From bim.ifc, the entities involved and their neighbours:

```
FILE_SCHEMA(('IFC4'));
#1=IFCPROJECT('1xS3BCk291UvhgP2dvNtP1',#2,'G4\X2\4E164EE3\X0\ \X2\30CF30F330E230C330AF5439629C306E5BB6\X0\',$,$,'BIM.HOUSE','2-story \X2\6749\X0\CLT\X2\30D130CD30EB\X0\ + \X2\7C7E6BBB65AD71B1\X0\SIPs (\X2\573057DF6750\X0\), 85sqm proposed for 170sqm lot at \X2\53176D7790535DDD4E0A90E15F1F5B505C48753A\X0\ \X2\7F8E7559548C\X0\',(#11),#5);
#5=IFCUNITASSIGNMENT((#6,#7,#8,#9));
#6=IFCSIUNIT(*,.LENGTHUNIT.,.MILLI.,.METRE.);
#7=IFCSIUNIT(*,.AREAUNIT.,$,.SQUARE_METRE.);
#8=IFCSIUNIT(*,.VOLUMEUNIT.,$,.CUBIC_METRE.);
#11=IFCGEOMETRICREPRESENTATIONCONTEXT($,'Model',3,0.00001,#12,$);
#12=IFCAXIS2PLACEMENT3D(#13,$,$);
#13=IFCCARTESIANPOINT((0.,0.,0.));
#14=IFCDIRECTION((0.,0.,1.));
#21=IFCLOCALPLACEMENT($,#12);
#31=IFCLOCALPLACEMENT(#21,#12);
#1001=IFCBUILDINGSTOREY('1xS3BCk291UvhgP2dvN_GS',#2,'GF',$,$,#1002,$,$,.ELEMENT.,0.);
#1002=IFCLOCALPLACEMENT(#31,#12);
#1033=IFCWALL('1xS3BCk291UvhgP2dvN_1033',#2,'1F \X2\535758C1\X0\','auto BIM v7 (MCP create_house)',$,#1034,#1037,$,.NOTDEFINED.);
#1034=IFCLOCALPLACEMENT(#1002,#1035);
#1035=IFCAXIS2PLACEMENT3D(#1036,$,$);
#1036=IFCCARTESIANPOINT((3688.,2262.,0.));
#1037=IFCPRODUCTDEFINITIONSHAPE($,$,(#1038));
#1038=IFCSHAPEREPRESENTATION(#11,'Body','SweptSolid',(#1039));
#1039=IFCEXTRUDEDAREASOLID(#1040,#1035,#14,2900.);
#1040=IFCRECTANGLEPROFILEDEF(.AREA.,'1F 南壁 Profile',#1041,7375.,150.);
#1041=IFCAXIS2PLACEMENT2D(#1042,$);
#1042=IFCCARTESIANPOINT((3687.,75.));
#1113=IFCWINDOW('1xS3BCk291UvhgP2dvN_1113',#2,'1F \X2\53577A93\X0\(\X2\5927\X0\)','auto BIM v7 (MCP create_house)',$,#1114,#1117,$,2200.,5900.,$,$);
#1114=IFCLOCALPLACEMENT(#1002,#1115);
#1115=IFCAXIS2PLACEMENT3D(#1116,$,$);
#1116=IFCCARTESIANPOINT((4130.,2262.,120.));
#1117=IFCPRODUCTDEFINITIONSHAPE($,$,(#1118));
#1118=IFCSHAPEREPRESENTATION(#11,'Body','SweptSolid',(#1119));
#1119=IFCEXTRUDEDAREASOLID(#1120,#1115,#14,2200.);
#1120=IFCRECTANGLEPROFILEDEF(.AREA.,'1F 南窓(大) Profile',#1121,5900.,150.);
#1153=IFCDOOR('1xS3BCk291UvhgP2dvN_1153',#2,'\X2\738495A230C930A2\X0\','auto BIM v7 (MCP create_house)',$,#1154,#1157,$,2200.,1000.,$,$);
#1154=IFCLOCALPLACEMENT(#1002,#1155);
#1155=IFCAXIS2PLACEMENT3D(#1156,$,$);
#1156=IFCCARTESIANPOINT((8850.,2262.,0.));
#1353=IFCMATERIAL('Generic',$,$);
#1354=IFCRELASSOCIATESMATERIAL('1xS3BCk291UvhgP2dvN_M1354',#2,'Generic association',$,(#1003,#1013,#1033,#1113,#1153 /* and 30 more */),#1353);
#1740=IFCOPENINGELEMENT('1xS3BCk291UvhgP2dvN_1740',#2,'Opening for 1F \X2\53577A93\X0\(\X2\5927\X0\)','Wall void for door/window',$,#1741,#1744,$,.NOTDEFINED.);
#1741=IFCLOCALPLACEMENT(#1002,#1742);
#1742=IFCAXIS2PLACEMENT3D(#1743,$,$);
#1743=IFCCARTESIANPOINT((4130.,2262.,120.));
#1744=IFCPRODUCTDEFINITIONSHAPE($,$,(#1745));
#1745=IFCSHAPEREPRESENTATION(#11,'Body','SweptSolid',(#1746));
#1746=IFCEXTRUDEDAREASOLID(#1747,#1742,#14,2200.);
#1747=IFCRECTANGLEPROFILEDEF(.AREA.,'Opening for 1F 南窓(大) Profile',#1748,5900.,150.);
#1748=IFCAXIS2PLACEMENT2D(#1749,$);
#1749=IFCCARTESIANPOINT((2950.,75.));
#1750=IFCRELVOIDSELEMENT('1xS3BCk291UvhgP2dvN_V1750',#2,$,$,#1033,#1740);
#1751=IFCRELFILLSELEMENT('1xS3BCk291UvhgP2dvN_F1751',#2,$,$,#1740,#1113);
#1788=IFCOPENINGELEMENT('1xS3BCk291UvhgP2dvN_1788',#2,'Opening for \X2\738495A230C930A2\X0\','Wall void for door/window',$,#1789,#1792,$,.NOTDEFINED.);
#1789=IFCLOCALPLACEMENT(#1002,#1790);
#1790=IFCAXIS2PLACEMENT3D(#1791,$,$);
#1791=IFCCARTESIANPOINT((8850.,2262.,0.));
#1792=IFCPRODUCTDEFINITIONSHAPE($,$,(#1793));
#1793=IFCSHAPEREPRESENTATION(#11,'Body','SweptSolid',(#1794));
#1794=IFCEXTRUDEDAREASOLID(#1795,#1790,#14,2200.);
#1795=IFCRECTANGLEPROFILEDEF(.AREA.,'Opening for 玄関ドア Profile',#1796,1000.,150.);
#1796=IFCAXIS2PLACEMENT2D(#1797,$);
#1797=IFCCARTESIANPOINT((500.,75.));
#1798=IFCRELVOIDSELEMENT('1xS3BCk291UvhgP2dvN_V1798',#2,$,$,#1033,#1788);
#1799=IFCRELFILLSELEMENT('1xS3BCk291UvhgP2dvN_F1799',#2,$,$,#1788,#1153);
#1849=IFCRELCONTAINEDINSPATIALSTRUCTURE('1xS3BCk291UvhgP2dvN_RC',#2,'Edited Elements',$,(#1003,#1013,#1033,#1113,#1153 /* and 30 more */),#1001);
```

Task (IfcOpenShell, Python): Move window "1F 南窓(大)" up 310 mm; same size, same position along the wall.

```python
import numpy as np
import ifcopenshell
import ifcopenshell.api.geometry
import ifcopenshell.util.placement
import ifcopenshell.util.unit

model = ifcopenshell.open("bim.ifc")
unit_scale = ifcopenshell.util.unit.calculate_unit_scale(model)

window = model.by_guid("1xS3BCk291UvhgP2dvN_1113")
opening = window.FillsVoids[0].RelatingOpeningElement
dz = 310.0

shift = np.array([0.0, 0.0, dz])
# The window is not placed relative to its opening, so move both.
for product in (opening, window):
    matrix = ifcopenshell.util.placement.get_local_placement(product.ObjectPlacement)
    matrix[:3, 3] += shift
    ifcopenshell.api.geometry.edit_object_placement(model, product=product, matrix=matrix, is_si=False)

print(f"moved by {dz * unit_scale:+.3f} m")

model.write("bim_edited.ifc")
```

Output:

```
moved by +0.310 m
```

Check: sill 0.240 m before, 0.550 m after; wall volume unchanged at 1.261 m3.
